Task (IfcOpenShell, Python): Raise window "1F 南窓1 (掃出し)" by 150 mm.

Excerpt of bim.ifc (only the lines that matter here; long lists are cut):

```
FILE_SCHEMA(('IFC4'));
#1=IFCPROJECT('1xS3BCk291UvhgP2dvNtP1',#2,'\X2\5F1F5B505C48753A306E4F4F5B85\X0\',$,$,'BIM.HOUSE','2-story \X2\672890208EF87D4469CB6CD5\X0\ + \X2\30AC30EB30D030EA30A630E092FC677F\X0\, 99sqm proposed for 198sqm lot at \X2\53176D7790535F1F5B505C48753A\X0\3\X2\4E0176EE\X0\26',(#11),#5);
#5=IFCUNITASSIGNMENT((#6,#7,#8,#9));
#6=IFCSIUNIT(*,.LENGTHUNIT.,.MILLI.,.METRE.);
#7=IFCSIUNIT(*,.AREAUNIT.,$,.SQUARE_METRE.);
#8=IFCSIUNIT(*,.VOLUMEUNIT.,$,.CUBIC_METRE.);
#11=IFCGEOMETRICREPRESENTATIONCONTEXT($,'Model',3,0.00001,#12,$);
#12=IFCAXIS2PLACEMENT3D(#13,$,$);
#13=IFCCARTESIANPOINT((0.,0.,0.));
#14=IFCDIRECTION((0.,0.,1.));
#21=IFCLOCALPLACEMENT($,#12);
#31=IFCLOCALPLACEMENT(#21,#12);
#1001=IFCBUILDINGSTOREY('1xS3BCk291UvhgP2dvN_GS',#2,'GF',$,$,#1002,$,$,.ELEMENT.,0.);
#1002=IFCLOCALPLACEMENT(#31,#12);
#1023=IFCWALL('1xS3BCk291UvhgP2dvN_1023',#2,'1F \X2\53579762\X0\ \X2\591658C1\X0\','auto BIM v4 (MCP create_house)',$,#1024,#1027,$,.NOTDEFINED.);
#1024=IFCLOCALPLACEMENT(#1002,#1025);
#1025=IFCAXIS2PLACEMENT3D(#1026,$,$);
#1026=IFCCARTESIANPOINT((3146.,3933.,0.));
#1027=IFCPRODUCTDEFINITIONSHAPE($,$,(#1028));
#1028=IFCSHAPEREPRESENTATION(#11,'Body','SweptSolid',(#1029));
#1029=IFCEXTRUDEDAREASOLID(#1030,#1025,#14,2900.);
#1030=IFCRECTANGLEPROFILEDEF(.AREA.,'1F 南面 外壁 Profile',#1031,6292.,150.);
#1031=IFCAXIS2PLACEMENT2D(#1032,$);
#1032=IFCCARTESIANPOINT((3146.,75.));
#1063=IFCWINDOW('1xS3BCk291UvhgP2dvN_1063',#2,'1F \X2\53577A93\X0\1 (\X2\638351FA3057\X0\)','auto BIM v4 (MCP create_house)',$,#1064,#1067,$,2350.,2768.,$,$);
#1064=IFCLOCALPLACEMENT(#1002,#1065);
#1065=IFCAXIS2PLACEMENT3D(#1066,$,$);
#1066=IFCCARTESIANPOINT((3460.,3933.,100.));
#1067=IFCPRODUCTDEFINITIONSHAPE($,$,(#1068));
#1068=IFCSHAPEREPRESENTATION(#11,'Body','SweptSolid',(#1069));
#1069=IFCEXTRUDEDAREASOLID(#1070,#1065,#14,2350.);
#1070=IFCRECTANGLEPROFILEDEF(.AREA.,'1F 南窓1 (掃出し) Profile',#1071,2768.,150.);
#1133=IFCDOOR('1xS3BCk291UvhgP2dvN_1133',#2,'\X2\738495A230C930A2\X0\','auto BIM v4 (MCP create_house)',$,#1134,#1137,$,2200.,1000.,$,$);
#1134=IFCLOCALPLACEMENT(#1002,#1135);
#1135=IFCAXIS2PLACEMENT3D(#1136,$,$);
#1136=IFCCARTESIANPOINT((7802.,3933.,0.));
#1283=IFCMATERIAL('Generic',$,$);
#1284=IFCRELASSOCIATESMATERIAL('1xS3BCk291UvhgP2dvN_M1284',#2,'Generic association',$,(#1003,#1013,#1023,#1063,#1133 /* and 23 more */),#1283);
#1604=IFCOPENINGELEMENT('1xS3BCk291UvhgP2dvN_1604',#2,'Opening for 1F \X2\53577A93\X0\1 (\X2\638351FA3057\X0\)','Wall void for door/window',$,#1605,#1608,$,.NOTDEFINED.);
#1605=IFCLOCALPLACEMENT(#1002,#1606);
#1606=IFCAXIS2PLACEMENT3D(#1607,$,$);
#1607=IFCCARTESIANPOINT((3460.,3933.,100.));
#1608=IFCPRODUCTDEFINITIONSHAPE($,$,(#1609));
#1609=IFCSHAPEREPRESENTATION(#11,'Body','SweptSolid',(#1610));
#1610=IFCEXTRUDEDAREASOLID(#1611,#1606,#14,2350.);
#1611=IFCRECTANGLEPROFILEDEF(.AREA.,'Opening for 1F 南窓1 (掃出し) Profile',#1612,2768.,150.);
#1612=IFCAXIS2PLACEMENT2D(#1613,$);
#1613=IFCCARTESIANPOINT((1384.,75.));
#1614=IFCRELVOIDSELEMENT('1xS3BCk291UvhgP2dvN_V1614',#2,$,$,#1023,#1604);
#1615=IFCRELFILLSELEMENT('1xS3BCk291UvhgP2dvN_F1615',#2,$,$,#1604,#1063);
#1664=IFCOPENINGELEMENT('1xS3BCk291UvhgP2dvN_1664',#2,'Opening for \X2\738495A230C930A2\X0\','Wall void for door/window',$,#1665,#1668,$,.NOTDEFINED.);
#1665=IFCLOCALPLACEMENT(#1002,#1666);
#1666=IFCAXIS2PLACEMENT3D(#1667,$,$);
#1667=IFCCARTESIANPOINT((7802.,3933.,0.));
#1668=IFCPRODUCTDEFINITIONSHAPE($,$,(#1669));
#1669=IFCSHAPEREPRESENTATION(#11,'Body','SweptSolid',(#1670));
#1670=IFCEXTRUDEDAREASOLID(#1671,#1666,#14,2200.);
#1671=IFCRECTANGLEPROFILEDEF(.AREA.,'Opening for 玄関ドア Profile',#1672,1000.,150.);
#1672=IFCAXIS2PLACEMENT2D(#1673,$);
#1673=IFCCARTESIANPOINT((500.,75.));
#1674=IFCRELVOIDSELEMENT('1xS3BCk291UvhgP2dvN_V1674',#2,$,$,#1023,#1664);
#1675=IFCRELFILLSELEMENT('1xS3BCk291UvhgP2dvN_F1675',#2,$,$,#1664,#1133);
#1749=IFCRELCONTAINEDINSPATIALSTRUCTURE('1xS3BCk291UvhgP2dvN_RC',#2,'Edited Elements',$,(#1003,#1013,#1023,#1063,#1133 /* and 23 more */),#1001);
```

```python
import numpy as np
import ifcopenshell
import ifcopenshell.api.geometry
import ifcopenshell.util.placement
import ifcopenshell.util.unit

model = ifcopenshell.open("bim.ifc")
unit_scale = ifcopenshell.util.unit.calculate_unit_scale(model)

window = model.by_guid("1xS3BCk291UvhgP2dvN_1063")
opening = window.FillsVoids[0].RelatingOpeningElement
dz = 0.15 / unit_scale

shift = np.array([0.0, 0.0, dz])
# The window is not placed relative to its opening, so move both.
for product in (opening, window):
    matrix = ifcopenshell.util.placement.get_local_placement(product.ObjectPlacement)
    matrix[:3, 3] += shift
    ifcopenshell.api.geometry.edit_object_placement(model, product=product, matrix=matrix, is_si=False)

print(f"moved by {dz * unit_scale:+.3f} m")

model.write("bim_edited.ifc")
```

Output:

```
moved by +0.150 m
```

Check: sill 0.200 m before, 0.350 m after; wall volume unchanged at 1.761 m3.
